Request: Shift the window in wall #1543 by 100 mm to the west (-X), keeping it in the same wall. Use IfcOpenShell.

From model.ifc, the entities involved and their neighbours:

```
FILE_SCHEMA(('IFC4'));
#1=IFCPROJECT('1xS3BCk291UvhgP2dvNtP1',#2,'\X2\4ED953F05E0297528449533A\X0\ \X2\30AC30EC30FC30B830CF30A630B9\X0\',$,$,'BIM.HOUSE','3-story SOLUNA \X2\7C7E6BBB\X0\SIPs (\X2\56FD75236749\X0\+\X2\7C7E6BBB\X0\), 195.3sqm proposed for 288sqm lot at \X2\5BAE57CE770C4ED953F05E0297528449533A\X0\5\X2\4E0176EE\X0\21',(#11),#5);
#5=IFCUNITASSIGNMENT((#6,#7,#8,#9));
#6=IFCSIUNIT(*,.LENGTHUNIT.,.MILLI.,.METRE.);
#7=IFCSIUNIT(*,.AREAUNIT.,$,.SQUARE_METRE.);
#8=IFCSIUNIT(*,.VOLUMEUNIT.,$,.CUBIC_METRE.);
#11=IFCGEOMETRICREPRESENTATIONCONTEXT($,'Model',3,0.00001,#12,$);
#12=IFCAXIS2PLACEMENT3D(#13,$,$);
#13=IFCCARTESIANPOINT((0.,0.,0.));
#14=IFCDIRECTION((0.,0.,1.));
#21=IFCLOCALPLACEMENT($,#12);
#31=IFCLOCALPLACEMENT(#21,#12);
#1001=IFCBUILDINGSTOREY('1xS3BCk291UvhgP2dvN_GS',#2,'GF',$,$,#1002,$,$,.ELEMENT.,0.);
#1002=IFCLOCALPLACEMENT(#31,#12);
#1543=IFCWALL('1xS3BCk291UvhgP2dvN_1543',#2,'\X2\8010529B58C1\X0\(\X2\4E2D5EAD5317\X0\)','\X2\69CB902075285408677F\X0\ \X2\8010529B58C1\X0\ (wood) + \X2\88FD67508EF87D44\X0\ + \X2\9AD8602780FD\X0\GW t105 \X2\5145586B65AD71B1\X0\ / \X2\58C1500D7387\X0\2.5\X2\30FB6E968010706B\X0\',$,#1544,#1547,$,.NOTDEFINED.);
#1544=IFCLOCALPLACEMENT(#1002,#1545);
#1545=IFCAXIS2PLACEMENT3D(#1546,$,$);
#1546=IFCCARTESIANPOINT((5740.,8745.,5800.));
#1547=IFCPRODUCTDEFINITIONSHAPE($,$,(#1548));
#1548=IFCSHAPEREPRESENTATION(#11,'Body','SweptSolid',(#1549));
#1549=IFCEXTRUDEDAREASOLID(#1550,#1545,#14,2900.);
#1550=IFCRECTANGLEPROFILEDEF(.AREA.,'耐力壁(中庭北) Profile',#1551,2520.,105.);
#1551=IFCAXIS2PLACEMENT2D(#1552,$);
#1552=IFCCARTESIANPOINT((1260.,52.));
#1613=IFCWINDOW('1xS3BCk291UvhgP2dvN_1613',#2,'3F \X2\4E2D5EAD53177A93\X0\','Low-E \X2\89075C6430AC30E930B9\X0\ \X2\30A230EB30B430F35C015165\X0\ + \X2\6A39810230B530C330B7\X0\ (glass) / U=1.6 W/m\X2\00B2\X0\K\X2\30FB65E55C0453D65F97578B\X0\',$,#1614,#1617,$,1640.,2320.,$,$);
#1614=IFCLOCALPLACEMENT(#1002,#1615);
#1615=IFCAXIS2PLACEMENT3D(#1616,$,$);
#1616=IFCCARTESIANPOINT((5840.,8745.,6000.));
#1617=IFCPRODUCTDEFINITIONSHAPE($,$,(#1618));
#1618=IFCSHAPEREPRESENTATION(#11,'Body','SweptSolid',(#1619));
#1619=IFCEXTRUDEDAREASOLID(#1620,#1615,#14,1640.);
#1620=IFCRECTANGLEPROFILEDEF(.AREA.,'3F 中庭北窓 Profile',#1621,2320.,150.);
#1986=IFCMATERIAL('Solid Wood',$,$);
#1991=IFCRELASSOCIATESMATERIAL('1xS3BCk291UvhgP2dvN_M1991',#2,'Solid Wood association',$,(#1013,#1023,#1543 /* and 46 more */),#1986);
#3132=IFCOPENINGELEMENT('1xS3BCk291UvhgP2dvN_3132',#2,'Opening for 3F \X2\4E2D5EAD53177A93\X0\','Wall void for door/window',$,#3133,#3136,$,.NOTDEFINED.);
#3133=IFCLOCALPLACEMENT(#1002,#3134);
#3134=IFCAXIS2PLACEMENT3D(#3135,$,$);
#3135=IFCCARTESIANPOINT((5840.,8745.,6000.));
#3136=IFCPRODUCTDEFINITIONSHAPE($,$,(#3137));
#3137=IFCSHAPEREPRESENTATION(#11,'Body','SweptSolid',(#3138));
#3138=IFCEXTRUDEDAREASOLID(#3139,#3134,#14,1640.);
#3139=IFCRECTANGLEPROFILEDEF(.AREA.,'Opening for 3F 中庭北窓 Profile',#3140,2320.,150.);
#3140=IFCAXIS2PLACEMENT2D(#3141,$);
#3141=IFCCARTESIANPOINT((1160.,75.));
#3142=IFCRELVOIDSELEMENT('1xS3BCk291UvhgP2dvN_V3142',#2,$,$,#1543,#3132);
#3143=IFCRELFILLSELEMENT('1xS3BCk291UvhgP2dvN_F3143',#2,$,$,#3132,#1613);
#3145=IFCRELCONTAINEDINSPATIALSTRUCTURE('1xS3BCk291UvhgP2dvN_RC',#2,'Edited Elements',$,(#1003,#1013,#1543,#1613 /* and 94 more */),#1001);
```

```python
import ifcopenshell
import ifcopenshell.api.geometry
import ifcopenshell.util.placement
import ifcopenshell.util.unit

model = ifcopenshell.open("model.ifc")
unit_scale = ifcopenshell.util.unit.calculate_unit_scale(model)

window = model.by_guid("1xS3BCk291UvhgP2dvN_1613")
opening = window.FillsVoids[0].RelatingOpeningElement
wall = opening.VoidsElements[0].RelatingBuildingElement

wall_matrix = ifcopenshell.util.placement.get_local_placement(wall.ObjectPlacement)
shift = wall_matrix[:3, 0] * -0.1 / unit_scale
before = ifcopenshell.util.placement.get_local_placement(window.ObjectPlacement)[:3, 3].copy()

# The window is not placed relative to its opening, so move both.
for product in (opening, window):
    matrix = ifcopenshell.util.placement.get_local_placement(product.ObjectPlacement)
    matrix[:3, 3] += shift
    ifcopenshell.api.geometry.edit_object_placement(model, product=product, matrix=matrix, is_si=False)

after = ifcopenshell.util.placement.get_local_placement(window.ObjectPlacement)[:3, 3]
print("window moved by", (after - before).round(3) + 0.0)

model.write("model_v2.ifc")
```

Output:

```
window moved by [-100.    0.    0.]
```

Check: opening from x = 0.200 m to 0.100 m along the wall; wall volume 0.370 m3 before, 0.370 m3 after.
